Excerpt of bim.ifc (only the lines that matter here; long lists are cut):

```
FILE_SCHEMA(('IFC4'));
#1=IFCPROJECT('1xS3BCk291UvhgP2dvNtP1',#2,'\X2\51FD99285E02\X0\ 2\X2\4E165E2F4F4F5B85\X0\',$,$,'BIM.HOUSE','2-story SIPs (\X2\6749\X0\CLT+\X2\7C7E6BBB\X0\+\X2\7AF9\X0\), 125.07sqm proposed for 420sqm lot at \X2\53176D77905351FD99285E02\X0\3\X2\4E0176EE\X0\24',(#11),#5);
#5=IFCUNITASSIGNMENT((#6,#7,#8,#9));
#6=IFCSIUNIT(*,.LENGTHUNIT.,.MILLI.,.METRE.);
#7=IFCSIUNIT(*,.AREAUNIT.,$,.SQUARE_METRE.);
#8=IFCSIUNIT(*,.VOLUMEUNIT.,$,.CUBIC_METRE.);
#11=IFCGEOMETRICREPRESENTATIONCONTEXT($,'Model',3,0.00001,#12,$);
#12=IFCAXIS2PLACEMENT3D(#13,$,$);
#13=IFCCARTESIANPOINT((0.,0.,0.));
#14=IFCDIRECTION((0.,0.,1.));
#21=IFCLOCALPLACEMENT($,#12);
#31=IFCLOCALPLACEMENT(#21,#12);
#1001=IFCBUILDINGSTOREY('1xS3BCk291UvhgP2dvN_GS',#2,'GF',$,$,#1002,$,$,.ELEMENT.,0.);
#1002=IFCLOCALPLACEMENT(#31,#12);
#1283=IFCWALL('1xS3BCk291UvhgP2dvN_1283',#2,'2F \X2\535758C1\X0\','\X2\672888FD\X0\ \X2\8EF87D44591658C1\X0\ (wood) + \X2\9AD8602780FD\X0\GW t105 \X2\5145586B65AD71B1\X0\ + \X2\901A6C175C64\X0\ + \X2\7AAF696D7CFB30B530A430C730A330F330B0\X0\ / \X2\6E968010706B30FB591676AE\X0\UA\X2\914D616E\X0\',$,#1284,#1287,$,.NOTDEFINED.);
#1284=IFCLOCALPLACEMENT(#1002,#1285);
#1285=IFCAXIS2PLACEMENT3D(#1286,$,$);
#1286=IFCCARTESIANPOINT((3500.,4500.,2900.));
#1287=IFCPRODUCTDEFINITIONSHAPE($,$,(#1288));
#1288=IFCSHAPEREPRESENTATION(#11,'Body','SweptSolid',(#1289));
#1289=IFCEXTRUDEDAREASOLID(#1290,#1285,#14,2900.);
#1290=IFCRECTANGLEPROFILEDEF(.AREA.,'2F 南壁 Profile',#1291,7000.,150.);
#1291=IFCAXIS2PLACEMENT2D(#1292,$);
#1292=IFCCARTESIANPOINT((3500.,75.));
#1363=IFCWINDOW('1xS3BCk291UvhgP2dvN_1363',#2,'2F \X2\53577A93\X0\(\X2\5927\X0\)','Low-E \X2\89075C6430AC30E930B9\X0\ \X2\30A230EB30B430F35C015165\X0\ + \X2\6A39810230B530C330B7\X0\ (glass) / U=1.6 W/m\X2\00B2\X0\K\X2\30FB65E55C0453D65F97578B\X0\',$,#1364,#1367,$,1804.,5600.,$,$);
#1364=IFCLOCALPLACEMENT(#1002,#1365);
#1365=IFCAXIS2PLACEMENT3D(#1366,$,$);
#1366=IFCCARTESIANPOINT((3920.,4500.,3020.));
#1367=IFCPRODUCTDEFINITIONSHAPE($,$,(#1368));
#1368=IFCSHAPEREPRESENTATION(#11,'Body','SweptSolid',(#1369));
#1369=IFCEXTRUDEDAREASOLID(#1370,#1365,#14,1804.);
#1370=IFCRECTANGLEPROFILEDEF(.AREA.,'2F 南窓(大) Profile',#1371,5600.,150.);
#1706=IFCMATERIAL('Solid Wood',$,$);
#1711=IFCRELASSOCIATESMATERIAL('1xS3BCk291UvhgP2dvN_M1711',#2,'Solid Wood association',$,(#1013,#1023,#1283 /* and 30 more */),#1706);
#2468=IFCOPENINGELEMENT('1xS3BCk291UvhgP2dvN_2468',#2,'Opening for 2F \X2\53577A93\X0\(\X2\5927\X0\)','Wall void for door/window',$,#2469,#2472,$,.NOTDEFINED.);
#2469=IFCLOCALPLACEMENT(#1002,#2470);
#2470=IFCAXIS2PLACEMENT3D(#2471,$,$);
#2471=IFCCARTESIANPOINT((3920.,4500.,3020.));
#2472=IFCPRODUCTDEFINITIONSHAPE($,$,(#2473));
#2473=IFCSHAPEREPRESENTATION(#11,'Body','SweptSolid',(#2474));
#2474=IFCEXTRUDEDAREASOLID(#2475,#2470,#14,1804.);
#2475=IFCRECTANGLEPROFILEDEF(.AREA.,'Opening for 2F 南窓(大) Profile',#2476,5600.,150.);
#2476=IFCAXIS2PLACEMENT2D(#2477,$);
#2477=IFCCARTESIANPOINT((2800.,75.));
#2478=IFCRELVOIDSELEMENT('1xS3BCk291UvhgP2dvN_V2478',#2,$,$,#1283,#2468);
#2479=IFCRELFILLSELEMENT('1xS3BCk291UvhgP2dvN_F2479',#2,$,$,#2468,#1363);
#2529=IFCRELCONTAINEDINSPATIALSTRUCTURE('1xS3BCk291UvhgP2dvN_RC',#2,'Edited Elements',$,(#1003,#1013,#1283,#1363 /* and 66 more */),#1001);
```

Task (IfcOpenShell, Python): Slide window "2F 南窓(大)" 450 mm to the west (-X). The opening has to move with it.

```python
import ifcopenshell
import ifcopenshell.api.geometry
import ifcopenshell.util.placement
import ifcopenshell.util.unit

model = ifcopenshell.open("bim.ifc")
unit_scale = ifcopenshell.util.unit.calculate_unit_scale(model)

window = model.by_guid("1xS3BCk291UvhgP2dvN_1363")
opening = window.FillsVoids[0].RelatingOpeningElement
wall = opening.VoidsElements[0].RelatingBuildingElement

wall_matrix = ifcopenshell.util.placement.get_local_placement(wall.ObjectPlacement)
shift = wall_matrix[:3, 0] * -0.45 / unit_scale
before = ifcopenshell.util.placement.get_local_placement(window.ObjectPlacement)[:3, 3].copy()

# The window is not placed relative to its opening, so move both.
for product in (opening, window):
    matrix = ifcopenshell.util.placement.get_local_placement(product.ObjectPlacement)
    matrix[:3, 3] += shift
    ifcopenshell.api.geometry.edit_object_placement(model, product=product, matrix=matrix, is_si=False)

after = ifcopenshell.util.placement.get_local_placement(window.ObjectPlacement)[:3, 3]
print("window moved by", (after - before).round(3) + 0.0)

model.write("bim_updated.ifc")
```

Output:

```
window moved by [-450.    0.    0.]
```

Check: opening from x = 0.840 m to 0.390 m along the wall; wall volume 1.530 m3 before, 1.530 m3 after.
